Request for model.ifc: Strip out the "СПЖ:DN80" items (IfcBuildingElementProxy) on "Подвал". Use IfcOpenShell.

First a look at what the model holds.

```python
import ifcopenshell
import ifcopenshell.util.element

model = ifcopenshell.open("model.ifc")
print(model.schema)
storey = next(s for s in model.by_type("IfcBuildingStorey") if s.Name == "Подвал")
proxies = [e for e in ifcopenshell.util.element.get_decomposition(storey) if e.is_a("IfcBuildingElementProxy")]
seen = {}
for e in proxies:
    element_type = ifcopenshell.util.element.get_type(e)
    name = element_type.Name if element_type not in (None, e) else None
    seen[name] = seen.get(name, 0) + 1
for name, count in sorted(seen.items(), key=str):
    print(count, "x", name)
```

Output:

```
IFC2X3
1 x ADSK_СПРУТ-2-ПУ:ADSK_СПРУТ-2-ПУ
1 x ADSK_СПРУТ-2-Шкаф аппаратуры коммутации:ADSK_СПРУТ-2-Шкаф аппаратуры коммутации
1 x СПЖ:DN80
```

```python
import ifcopenshell
import ifcopenshell.api.root
import ifcopenshell.util.element

model = ifcopenshell.open("model.ifc")

storey = next(s for s in model.by_type("IfcBuildingStorey") if s.Name == "Подвал")
proxies = [e for e in ifcopenshell.util.element.get_decomposition(storey) if e.is_a("IfcBuildingElementProxy")]
targets = [e for e in proxies if (t := ifcopenshell.util.element.get_type(e)) not in (None, e) and t.Name == "СПЖ:DN80"]

for e in targets:
    ifcopenshell.api.root.remove_product(model, product=e)
print(len(targets), "removed")

model.write("model_rev.ifc")
```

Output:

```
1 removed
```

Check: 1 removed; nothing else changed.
